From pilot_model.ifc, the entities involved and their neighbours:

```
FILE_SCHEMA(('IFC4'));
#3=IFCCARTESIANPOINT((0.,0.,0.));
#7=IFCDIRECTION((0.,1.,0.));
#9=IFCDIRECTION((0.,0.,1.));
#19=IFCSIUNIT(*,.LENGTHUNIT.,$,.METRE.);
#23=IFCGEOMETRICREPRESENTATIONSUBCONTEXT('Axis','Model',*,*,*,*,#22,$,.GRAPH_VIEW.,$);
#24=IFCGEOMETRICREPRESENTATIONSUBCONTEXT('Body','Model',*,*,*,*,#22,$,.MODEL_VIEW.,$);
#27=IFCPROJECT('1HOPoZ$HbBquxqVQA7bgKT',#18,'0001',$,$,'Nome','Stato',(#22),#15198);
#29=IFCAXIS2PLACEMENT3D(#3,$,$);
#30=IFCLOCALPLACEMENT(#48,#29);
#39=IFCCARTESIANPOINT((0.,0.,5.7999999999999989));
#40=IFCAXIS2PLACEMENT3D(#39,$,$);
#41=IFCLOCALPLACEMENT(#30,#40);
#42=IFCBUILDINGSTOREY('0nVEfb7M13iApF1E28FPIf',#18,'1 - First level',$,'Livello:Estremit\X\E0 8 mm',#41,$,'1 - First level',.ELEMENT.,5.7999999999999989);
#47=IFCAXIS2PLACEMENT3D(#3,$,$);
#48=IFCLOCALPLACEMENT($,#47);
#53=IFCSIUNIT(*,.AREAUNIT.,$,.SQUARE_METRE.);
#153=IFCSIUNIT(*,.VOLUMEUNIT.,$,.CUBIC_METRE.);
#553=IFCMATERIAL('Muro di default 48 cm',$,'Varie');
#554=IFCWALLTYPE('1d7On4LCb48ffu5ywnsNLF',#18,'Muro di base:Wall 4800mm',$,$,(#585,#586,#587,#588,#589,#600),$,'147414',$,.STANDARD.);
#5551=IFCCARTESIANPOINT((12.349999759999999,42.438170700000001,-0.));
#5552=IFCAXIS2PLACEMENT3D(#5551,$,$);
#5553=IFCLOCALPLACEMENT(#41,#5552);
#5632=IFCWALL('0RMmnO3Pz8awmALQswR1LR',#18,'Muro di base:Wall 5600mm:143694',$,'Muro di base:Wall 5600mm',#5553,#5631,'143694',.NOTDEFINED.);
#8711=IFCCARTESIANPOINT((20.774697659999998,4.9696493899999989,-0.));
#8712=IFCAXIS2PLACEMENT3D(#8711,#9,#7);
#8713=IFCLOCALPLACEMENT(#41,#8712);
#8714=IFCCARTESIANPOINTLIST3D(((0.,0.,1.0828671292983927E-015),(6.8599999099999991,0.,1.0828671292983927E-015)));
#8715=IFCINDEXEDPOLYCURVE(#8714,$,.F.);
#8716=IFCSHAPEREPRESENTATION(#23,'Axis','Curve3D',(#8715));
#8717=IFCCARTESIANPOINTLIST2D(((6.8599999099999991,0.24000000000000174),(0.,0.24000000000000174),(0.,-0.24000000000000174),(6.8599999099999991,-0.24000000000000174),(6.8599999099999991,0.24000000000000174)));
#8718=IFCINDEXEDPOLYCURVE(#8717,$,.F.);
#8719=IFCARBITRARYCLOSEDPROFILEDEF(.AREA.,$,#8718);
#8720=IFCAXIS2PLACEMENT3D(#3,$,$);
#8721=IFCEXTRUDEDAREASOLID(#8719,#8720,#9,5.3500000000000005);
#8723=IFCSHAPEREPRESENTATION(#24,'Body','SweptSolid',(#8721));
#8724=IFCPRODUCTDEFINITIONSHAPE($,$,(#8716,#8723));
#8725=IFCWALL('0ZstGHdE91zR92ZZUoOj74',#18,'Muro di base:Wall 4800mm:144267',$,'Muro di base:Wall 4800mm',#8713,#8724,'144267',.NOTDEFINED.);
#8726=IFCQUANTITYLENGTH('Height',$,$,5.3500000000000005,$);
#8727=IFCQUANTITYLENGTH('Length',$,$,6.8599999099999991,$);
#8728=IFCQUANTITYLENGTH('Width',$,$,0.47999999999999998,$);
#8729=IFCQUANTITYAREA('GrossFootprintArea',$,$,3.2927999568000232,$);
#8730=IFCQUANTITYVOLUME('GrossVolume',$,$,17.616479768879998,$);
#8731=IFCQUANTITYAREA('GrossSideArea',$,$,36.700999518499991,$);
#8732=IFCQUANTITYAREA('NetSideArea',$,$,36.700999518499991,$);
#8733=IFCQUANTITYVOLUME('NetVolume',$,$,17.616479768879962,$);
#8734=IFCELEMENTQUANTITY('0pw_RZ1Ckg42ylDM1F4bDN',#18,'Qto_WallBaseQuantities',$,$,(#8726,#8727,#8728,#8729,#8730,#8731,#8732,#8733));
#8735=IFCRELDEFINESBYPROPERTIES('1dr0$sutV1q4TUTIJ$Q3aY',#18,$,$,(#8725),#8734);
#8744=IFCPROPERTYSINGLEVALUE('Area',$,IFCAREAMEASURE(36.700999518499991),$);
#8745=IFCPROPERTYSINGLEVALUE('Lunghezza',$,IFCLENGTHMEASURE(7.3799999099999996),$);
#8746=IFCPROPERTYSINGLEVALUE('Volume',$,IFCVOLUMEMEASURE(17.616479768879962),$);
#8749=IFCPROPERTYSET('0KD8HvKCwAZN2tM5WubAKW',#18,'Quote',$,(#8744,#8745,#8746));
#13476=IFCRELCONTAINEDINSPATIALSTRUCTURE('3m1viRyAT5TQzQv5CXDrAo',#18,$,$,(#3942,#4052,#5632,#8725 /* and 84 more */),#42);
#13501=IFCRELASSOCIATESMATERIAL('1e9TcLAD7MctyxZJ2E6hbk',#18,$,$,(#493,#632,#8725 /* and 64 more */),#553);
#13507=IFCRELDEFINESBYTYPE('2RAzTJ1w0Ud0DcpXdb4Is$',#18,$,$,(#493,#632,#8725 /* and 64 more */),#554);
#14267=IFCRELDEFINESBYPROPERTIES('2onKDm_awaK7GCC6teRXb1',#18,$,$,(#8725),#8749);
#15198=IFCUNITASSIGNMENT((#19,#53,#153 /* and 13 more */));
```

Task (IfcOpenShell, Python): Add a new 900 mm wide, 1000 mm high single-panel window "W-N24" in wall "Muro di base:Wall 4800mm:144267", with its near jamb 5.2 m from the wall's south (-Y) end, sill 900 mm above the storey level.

```python
import numpy as np
import ifcopenshell
import ifcopenshell.api.feature
import ifcopenshell.api.geometry
import ifcopenshell.api.pset
import ifcopenshell.api.root
import ifcopenshell.api.spatial
import ifcopenshell.geom
import ifcopenshell.util.element
import ifcopenshell.util.placement
import ifcopenshell.util.representation
import ifcopenshell.util.shape
import ifcopenshell.util.unit

model = ifcopenshell.open("pilot_model.ifc")
unit_scale = ifcopenshell.util.unit.calculate_unit_scale(model)
area_scale = ifcopenshell.util.unit.calculate_unit_scale(model, "AREAUNIT")
volume_scale = ifcopenshell.util.unit.calculate_unit_scale(model, "VOLUMEUNIT")
settings = ifcopenshell.geom.settings()


def volume(element):
    """Net volume in cubic metres, openings subtracted."""
    shape = ifcopenshell.geom.create_shape(settings, element)
    return ifcopenshell.util.shape.get_volume(shape.geometry)


wall = model.by_guid("0ZstGHdE91zR92ZZUoOj74")
storey = ifcopenshell.util.element.get_container(wall, ifc_class="IfcBuildingStorey")
context = ifcopenshell.util.representation.get_context(model, "Model", "Body", "MODEL_VIEW")
before = volume(wall)

width, height, from_end, sill = 0.9, 1, 5.2, 0.9  # metres

# The wall runs along its own X axis, and the end named is its -X end.
wall_shape = ifcopenshell.geom.create_shape(settings, wall)
x, y, z = ifcopenshell.util.shape.get_vertices(wall_shape.geometry).T
start = x.min() + from_end
face, thickness = float(y.min()), float(y.max() - y.min())
wall_matrix = ifcopenshell.util.placement.get_local_placement(wall.ObjectPlacement)
level = ifcopenshell.util.placement.get_local_placement(storey.ObjectPlacement)[2, 3]


def in_wall(x, y):
    """Placement at x, y metres in the wall's axes, at sill height."""
    matrix = wall_matrix.copy()
    matrix[:, 3] = wall_matrix @ np.array([x / unit_scale, y / unit_scale, 0.0, 1.0])
    matrix[2, 3] = level + sill / unit_scale
    return matrix


# Opening: a box that overshoots both wall faces by 50 mm.
opening = ifcopenshell.api.root.create_entity(model, ifc_class="IfcOpeningElement", predefined_type="OPENING")
box = ifcopenshell.api.geometry.add_wall_representation(
    model, context=context, length=width, height=height, thickness=thickness + 0.1
)
ifcopenshell.api.geometry.assign_representation(model, product=opening, representation=box)
ifcopenshell.api.geometry.edit_object_placement(model, product=opening, matrix=in_wall(start, face - 0.05), is_si=False)
ifcopenshell.api.feature.add_feature(model, feature=opening, element=wall)

window = ifcopenshell.api.root.create_entity(model, ifc_class="IfcWindow", name="W-N24", predefined_type="WINDOW")
window.OverallWidth, window.OverallHeight = width / unit_scale, height / unit_scale
window.PartitioningType = "SINGLE_PANEL"
body = ifcopenshell.api.geometry.add_window_representation(
    model,
    context=context,
    overall_width=window.OverallWidth,
    overall_height=window.OverallHeight,
    partition_type="SINGLE_PANEL",
)
ifcopenshell.api.geometry.assign_representation(model, product=window, representation=body)
ifcopenshell.api.spatial.assign_container(model, products=[window], relating_structure=storey)
ifcopenshell.api.feature.add_filling(model, opening=opening, element=window)

# Centre the window in the wall's thickness.
ifcopenshell.api.geometry.edit_object_placement(model, product=window, matrix=in_wall(start, face), is_si=False)
window_shape = ifcopenshell.geom.create_shape(settings, window)
depth = ifcopenshell.util.shape.get_vertices(window_shape.geometry)[:, 1]
offset = face + thickness / 2 - (depth.min() + depth.max()) / 2
ifcopenshell.api.geometry.edit_object_placement(model, product=window, matrix=in_wall(start, offset), is_si=False)

after = volume(wall)

# Update the wall's stored quantities.
qto = model.by_id(ifcopenshell.util.element.get_pset(wall, "Qto_WallBaseQuantities", should_inherit=False)["id"])
ifcopenshell.api.pset.edit_qto(model, qto=qto, properties={
    "NetSideArea": after / thickness / area_scale,
    "NetVolume": after / volume_scale,
})
pset = model.by_id(ifcopenshell.util.element.get_pset(wall, "Quote", should_inherit=False)["id"])
ifcopenshell.api.pset.edit_pset(model, pset=pset, properties={
    "Area": model.create_entity("IfcAreaMeasure", after / thickness / area_scale),
    "Volume": model.create_entity("IfcVolumeMeasure", after / volume_scale),
})

print(f"wall volume {before:.3f} -> {after:.3f} m3")

model.write("pilot_model_edited.ifc")
```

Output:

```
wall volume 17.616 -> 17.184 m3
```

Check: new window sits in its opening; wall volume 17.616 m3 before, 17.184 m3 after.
